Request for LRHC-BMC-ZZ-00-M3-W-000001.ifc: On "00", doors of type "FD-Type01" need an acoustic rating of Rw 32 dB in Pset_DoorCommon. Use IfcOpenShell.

First a look at what the model holds.

```python
import ifcopenshell
import ifcopenshell.util.element

model = ifcopenshell.open("LRHC-BMC-ZZ-00-M3-W-000001.ifc")
print(model.schema)
storey = next(s for s in model.by_type("IfcBuildingStorey") if s.Name == "00")
doors = [e for e in ifcopenshell.util.element.get_decomposition(storey) if e.is_a("IfcDoor")]
seen = {}
for e in doors:
    element_type = ifcopenshell.util.element.get_type(e)
    key = (element_type.Name if element_type != e and element_type else None, ifcopenshell.util.element.get_pset(e, "Pset_DoorCommon", "AcousticRating"))
    seen[key] = seen.get(key, 0) + 1
for (name, value), count in sorted(seen.items(), key=str):
    print(count, "x", name, "|", value)
```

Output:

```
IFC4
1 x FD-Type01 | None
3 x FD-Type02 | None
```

```python
import ifcopenshell
import ifcopenshell.api.pset
import ifcopenshell.util.element

model = ifcopenshell.open("LRHC-BMC-ZZ-00-M3-W-000001.ifc")

storey = next(s for s in model.by_type("IfcBuildingStorey") if s.Name == "00")
doors = [e for e in ifcopenshell.util.element.get_decomposition(storey) if e.is_a("IfcDoor")]

count = 0
for e in doors:
    element_type = ifcopenshell.util.element.get_type(e)
    if element_type in (None, e) or element_type.Name != "FD-Type01":
        continue
    # add_pset returns the element's existing set when there is one.
    pset = ifcopenshell.api.pset.add_pset(model, product=e, name="Pset_DoorCommon")
    ifcopenshell.api.pset.edit_pset(model, pset=pset, properties={"AcousticRating": "Rw 32 dB"})
    count += 1

print(count, "doors updated")

model.write("LRHC-BMC-ZZ-00-M3-W-000001_v2.ifc")
```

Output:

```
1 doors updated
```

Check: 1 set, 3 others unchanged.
